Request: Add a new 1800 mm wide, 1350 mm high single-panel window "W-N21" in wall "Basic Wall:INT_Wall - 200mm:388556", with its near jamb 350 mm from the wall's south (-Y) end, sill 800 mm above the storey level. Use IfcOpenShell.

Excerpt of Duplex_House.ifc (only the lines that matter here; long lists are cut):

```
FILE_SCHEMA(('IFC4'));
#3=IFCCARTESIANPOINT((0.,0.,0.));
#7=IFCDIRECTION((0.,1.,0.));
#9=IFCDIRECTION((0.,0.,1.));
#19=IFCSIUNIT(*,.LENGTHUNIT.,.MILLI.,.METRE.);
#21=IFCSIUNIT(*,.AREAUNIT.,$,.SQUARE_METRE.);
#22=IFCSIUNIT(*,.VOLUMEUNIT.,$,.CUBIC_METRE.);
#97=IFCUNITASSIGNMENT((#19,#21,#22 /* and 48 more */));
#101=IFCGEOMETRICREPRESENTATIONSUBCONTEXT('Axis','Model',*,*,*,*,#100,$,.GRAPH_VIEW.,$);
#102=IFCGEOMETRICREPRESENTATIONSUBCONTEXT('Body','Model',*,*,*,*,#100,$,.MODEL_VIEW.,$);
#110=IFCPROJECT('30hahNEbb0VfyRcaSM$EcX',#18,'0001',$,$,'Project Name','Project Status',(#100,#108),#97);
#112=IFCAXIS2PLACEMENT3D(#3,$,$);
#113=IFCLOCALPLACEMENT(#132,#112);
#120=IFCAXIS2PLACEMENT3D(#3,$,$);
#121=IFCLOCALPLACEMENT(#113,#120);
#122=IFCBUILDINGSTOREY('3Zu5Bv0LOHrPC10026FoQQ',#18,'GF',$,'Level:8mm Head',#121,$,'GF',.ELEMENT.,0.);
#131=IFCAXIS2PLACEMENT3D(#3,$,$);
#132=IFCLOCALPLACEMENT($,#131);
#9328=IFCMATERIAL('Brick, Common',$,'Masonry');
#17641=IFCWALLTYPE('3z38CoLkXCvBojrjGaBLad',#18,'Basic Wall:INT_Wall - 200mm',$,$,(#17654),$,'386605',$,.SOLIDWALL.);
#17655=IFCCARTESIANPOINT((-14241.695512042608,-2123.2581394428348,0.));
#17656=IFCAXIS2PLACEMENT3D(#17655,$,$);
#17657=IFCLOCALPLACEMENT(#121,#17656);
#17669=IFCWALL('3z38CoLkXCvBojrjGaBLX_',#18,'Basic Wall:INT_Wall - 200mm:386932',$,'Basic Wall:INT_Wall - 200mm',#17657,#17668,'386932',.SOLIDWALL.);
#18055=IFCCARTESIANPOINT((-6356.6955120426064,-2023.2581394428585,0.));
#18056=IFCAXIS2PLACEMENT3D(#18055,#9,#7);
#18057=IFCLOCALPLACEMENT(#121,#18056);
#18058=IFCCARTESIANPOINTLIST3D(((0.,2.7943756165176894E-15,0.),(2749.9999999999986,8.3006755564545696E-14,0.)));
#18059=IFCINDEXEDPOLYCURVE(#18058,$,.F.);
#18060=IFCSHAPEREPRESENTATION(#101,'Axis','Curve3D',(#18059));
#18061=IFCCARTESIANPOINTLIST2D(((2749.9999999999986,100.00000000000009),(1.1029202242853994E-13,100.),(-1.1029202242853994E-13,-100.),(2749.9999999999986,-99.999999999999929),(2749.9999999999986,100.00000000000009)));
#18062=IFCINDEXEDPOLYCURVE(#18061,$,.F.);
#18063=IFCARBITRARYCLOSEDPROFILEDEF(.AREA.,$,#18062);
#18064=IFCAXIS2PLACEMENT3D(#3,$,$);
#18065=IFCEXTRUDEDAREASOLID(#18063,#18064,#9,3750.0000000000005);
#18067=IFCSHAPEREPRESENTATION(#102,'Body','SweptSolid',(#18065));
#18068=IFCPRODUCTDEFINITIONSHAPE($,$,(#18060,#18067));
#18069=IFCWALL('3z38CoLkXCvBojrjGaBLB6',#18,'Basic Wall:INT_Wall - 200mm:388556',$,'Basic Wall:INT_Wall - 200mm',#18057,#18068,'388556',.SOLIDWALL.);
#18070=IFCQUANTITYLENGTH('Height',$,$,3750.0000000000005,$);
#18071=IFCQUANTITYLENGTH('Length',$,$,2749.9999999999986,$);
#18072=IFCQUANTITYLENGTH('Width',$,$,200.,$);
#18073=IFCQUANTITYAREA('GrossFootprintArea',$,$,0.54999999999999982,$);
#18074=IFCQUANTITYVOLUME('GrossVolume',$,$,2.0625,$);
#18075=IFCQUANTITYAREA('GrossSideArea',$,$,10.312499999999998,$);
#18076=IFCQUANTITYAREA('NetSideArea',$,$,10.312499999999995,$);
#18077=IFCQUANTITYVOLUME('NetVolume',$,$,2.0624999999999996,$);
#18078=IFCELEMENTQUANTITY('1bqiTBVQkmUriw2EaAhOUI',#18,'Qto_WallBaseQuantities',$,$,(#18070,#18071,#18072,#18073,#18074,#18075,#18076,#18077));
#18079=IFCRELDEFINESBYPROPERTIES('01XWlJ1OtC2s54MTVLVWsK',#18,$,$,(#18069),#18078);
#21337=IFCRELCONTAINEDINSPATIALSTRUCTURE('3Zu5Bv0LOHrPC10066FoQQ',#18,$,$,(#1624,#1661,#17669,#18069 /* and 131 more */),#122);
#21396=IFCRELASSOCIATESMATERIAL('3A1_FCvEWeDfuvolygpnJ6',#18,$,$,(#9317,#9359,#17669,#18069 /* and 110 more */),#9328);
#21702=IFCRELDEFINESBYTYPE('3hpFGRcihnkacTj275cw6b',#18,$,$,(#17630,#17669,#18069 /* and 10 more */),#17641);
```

```python
import numpy as np
import ifcopenshell
import ifcopenshell.api.feature
import ifcopenshell.api.geometry
import ifcopenshell.api.pset
import ifcopenshell.api.root
import ifcopenshell.api.spatial
import ifcopenshell.geom
import ifcopenshell.util.element
import ifcopenshell.util.placement
import ifcopenshell.util.representation
import ifcopenshell.util.shape
import ifcopenshell.util.unit

model = ifcopenshell.open("Duplex_House.ifc")
unit_scale = ifcopenshell.util.unit.calculate_unit_scale(model)
area_scale = ifcopenshell.util.unit.calculate_unit_scale(model, "AREAUNIT")
volume_scale = ifcopenshell.util.unit.calculate_unit_scale(model, "VOLUMEUNIT")
settings = ifcopenshell.geom.settings()


def volume(element):
    """Net volume in cubic metres, openings subtracted."""
    shape = ifcopenshell.geom.create_shape(settings, element)
    return ifcopenshell.util.shape.get_volume(shape.geometry)


wall = model.by_guid("3z38CoLkXCvBojrjGaBLB6")
storey = ifcopenshell.util.element.get_container(wall, ifc_class="IfcBuildingStorey")
context = ifcopenshell.util.representation.get_context(model, "Model", "Body", "MODEL_VIEW")
before = volume(wall)

width, height, from_end, sill = 1.8, 1.35, 0.35, 0.8  # metres

# The wall runs along its own X axis, and the end named is its -X end.
wall_shape = ifcopenshell.geom.create_shape(settings, wall)
x, y, z = ifcopenshell.util.shape.get_vertices(wall_shape.geometry).T
start = x.min() + from_end
face, thickness = float(y.min()), float(y.max() - y.min())
wall_matrix = ifcopenshell.util.placement.get_local_placement(wall.ObjectPlacement)
level = ifcopenshell.util.placement.get_local_placement(storey.ObjectPlacement)[2, 3]


def in_wall(x, y):
    """Placement at x, y metres in the wall's axes, at sill height."""
    matrix = wall_matrix.copy()
    matrix[:, 3] = wall_matrix @ np.array([x / unit_scale, y / unit_scale, 0.0, 1.0])
    matrix[2, 3] = level + sill / unit_scale
    return matrix


# Opening: a box that overshoots both wall faces by 50 mm.
opening = ifcopenshell.api.root.create_entity(model, ifc_class="IfcOpeningElement", predefined_type="OPENING")
box = ifcopenshell.api.geometry.add_wall_representation(
    model, context=context, length=width, height=height, thickness=thickness + 0.1
)
ifcopenshell.api.geometry.assign_representation(model, product=opening, representation=box)
ifcopenshell.api.geometry.edit_object_placement(model, product=opening, matrix=in_wall(start, face - 0.05), is_si=False)
ifcopenshell.api.feature.add_feature(model, feature=opening, element=wall)

window = ifcopenshell.api.root.create_entity(model, ifc_class="IfcWindow", name="W-N21", predefined_type="WINDOW")
window.OverallWidth, window.OverallHeight = width / unit_scale, height / unit_scale
window.PartitioningType = "SINGLE_PANEL"
body = ifcopenshell.api.geometry.add_window_representation(
    model,
    context=context,
    overall_width=window.OverallWidth,
    overall_height=window.OverallHeight,
    partition_type="SINGLE_PANEL",
)
ifcopenshell.api.geometry.assign_representation(model, product=window, representation=body)
ifcopenshell.api.spatial.assign_container(model, products=[window], relating_structure=storey)
ifcopenshell.api.feature.add_filling(model, opening=opening, element=window)

# Centre the window in the wall's thickness.
ifcopenshell.api.geometry.edit_object_placement(model, product=window, matrix=in_wall(start, face), is_si=False)
window_shape = ifcopenshell.geom.create_shape(settings, window)
depth = ifcopenshell.util.shape.get_vertices(window_shape.geometry)[:, 1]
offset = face + thickness / 2 - (depth.min() + depth.max()) / 2
ifcopenshell.api.geometry.edit_object_placement(model, product=window, matrix=in_wall(start, offset), is_si=False)

after = volume(wall)

# Update the wall's stored quantities.
qto = model.by_id(ifcopenshell.util.element.get_pset(wall, "Qto_WallBaseQuantities", should_inherit=False)["id"])
ifcopenshell.api.pset.edit_qto(model, qto=qto, properties={
    "NetSideArea": after / thickness / area_scale,
    "NetVolume": after / volume_scale,
})

print(f"wall volume {before:.3f} -> {after:.3f} m3")

model.write("Duplex_House-out.ifc")
```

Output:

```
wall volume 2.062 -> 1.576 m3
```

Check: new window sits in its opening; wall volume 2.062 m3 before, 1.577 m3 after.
